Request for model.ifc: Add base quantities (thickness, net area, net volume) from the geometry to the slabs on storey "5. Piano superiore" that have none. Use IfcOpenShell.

First a look at what the model holds.

```python
import ifcopenshell
import ifcopenshell.util.element
import ifcopenshell.util.unit

model = ifcopenshell.open("model.ifc")
print(model.schema)
for unit_type in ("LENGTHUNIT", "AREAUNIT", "VOLUMEUNIT"):
    print(unit_type, ifcopenshell.util.unit.calculate_unit_scale(model, unit_type))
storey = next(s for s in model.by_type("IfcBuildingStorey") if s.Name == "5. Piano superiore")
slabs = [e for e in ifcopenshell.util.element.get_decomposition(storey) if e.is_a("IfcSlab")]
for e in sorted(slabs, key=lambda e: e.id()):
    print(e.id(), e.is_a(), e.Name, list(ifcopenshell.util.element.get_psets(e, qtos_only=True)), sep=" | ")
```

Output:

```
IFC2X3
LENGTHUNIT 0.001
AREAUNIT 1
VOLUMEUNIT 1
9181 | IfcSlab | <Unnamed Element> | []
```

```python
import ifcopenshell
import ifcopenshell.api.pset
import ifcopenshell.geom
import ifcopenshell.util.element
import ifcopenshell.util.shape
import ifcopenshell.util.unit

model = ifcopenshell.open("model.ifc")
unit_scale = ifcopenshell.util.unit.calculate_unit_scale(model)
area_scale = ifcopenshell.util.unit.calculate_unit_scale(model, "AREAUNIT")
volume_scale = ifcopenshell.util.unit.calculate_unit_scale(model, "VOLUMEUNIT")
settings = ifcopenshell.geom.settings()

storey = next(s for s in model.by_type("IfcBuildingStorey") if s.Name == "5. Piano superiore")
slabs = [e for e in ifcopenshell.util.element.get_decomposition(storey) if e.is_a("IfcSlab")]

for e in sorted(slabs, key=lambda e: e.id()):
    if ifcopenshell.util.element.get_psets(e, qtos_only=True, should_inherit=False):
        continue
    # Geometry comes back in metres, in the element's own axes.
    shape = ifcopenshell.geom.create_shape(settings, e)
    values = {
        "Width": ifcopenshell.util.shape.get_z(shape.geometry) / unit_scale,
        "NetArea": ifcopenshell.util.shape.get_footprint_area(shape.geometry) / area_scale,
        "NetVolume": ifcopenshell.util.shape.get_volume(shape.geometry) / volume_scale,
    }
    qto = ifcopenshell.api.pset.add_qto(model, product=e, name="BaseQuantities")
    ifcopenshell.api.pset.edit_qto(model, qto=qto, properties=values)
    print(e.id(), {k: round(v, 3) for k, v in values.items()})

model.write("model_edited.ifc")
```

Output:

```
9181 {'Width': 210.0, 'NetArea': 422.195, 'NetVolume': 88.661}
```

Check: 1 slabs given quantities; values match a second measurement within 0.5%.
